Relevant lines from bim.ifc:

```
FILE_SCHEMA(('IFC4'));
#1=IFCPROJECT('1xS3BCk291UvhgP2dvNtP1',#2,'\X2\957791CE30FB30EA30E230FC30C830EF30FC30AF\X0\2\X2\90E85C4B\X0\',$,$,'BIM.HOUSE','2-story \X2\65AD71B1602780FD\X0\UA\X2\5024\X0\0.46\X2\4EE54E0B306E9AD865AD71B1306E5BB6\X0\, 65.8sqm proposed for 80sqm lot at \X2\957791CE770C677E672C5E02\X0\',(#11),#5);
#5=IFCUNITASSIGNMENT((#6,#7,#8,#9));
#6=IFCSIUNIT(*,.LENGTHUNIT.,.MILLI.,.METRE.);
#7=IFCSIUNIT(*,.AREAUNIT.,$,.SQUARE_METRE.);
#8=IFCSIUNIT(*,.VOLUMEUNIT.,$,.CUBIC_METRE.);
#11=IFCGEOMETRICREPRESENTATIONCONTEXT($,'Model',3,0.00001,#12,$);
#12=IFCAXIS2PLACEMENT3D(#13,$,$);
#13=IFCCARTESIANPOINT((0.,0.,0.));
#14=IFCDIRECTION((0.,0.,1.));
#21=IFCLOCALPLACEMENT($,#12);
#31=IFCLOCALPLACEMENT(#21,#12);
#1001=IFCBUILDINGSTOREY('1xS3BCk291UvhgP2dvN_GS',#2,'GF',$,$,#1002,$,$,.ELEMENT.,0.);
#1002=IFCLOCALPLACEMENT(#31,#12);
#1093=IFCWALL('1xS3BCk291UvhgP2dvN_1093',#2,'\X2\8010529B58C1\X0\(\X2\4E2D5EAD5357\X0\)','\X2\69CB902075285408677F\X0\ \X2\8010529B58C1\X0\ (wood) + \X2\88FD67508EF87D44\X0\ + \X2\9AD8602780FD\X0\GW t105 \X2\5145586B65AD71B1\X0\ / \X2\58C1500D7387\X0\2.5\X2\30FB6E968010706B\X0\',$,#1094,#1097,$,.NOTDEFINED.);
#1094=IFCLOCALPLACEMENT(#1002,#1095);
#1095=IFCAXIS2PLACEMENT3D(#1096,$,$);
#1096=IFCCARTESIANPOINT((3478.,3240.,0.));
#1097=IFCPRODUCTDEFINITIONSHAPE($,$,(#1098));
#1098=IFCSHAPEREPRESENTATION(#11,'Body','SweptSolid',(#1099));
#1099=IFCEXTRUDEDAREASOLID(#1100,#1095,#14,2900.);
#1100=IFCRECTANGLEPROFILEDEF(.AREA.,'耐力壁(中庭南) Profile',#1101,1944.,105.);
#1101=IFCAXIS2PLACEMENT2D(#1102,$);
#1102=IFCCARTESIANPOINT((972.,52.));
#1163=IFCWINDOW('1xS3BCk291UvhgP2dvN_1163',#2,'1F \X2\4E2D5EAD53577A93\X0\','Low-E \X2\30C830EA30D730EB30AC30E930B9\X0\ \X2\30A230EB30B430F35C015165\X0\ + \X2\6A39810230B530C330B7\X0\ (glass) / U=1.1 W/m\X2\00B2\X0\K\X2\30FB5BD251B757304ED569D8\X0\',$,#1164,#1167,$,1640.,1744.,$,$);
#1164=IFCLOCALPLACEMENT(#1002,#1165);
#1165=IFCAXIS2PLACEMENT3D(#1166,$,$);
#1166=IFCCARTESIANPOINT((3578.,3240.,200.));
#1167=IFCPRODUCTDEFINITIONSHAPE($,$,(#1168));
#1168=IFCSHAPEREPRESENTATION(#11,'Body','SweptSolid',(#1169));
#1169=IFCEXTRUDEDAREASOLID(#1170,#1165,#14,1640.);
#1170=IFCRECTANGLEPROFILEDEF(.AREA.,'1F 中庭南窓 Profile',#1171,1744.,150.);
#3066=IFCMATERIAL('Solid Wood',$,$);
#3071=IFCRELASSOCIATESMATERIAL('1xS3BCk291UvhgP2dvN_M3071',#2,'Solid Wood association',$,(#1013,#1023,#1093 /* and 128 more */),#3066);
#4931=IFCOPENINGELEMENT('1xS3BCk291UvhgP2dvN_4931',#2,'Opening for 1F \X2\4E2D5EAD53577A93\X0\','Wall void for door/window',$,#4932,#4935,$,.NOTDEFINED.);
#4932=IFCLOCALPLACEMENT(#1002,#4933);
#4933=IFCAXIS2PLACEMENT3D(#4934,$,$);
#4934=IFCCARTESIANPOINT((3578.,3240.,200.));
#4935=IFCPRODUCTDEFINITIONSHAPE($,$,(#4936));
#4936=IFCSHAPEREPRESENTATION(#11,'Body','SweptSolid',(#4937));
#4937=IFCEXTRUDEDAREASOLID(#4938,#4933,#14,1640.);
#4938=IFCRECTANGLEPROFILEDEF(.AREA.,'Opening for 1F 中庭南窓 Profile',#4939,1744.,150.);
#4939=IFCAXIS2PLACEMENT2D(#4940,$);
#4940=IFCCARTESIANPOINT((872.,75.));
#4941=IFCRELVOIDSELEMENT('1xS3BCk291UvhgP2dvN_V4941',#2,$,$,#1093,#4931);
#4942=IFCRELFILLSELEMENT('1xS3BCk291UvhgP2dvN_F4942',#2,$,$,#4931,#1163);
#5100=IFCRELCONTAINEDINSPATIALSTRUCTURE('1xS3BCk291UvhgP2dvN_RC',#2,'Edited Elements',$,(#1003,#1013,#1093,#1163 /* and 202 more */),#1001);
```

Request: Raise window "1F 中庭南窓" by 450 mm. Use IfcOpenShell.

```python
import numpy as np
import ifcopenshell
import ifcopenshell.api.geometry
import ifcopenshell.util.placement
import ifcopenshell.util.unit

model = ifcopenshell.open("bim.ifc")
unit_scale = ifcopenshell.util.unit.calculate_unit_scale(model)

window = model.by_guid("1xS3BCk291UvhgP2dvN_1163")
opening = window.FillsVoids[0].RelatingOpeningElement
dz = 0.45 / unit_scale

shift = np.array([0.0, 0.0, dz])
# The window is not placed relative to its opening, so move both.
for product in (opening, window):
    matrix = ifcopenshell.util.placement.get_local_placement(product.ObjectPlacement)
    matrix[:3, 3] += shift
    ifcopenshell.api.geometry.edit_object_placement(model, product=product, matrix=matrix, is_si=False)

print(f"moved by {dz * unit_scale:+.3f} m")

model.write("bim_updated.ifc")
```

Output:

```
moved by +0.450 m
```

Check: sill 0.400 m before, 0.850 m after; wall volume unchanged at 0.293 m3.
